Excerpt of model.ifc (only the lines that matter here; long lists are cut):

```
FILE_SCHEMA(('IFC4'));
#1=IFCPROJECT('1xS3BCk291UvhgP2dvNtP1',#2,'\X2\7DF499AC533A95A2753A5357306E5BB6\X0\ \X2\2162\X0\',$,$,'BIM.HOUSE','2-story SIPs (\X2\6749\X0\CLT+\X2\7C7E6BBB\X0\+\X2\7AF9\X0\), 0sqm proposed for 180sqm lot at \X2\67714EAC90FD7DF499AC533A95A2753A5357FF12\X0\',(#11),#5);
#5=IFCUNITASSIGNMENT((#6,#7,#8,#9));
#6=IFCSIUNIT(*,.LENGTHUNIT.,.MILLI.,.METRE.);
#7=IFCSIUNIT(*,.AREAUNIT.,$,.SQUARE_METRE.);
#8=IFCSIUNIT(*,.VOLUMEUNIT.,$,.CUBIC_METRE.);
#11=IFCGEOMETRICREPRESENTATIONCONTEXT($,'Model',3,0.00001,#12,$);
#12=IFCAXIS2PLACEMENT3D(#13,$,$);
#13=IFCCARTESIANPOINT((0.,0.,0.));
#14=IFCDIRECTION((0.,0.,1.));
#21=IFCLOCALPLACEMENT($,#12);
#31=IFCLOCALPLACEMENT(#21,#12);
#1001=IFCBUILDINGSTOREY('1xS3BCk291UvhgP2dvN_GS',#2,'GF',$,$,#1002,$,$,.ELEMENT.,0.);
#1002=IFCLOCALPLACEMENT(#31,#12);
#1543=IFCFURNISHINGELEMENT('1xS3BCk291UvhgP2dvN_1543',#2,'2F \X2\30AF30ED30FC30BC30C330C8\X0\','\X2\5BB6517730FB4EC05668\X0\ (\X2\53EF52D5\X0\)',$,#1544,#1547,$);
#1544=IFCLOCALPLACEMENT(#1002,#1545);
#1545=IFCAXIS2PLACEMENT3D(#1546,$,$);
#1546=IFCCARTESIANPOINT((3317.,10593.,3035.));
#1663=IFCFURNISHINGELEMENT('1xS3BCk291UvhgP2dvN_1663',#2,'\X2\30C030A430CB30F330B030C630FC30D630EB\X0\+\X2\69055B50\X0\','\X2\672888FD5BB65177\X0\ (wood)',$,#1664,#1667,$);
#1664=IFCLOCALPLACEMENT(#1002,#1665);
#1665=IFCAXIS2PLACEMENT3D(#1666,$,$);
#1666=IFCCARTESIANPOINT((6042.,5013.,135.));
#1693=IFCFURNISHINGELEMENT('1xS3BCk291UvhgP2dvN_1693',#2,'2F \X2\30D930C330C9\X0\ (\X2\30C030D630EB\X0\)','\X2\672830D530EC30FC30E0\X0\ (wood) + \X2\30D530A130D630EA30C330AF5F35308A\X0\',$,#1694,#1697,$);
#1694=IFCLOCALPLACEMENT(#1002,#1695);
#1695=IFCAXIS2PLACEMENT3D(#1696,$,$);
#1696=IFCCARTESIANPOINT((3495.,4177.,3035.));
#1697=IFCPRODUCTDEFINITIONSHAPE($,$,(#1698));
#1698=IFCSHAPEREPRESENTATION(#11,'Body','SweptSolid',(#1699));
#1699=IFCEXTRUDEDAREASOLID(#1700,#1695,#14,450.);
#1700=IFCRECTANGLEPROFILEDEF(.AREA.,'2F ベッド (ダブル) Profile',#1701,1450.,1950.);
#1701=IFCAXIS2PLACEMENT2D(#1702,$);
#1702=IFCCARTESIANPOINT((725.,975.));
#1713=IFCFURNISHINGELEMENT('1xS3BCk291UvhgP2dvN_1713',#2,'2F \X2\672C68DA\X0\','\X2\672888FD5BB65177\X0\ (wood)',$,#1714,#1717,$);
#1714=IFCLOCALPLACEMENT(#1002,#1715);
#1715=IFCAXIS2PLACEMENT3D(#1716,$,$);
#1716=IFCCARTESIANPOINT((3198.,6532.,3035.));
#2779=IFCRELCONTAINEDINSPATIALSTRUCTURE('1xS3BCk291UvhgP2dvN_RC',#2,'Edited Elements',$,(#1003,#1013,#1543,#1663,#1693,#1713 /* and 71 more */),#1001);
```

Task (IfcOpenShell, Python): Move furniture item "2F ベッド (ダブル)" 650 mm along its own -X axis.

```python
import ifcopenshell
import ifcopenshell.api.geometry
import ifcopenshell.util.placement
import ifcopenshell.util.unit

model = ifcopenshell.open("model.ifc")
unit_scale = ifcopenshell.util.unit.calculate_unit_scale(model)

item = model.by_guid("1xS3BCk291UvhgP2dvN_1693")
matrix = ifcopenshell.util.placement.get_local_placement(item.ObjectPlacement)
matrix[:3, 3] -= matrix[:3, 0] * 0.65 / unit_scale
ifcopenshell.api.geometry.edit_object_placement(model, product=item, matrix=matrix, is_si=False)

print(ifcopenshell.util.placement.get_local_placement(item.ObjectPlacement).round(3) + 0.0)

model.write("model-out.ifc")
```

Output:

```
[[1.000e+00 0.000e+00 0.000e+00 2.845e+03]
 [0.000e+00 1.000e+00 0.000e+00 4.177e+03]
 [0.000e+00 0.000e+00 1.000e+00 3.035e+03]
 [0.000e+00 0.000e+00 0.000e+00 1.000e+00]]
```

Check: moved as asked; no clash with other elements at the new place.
